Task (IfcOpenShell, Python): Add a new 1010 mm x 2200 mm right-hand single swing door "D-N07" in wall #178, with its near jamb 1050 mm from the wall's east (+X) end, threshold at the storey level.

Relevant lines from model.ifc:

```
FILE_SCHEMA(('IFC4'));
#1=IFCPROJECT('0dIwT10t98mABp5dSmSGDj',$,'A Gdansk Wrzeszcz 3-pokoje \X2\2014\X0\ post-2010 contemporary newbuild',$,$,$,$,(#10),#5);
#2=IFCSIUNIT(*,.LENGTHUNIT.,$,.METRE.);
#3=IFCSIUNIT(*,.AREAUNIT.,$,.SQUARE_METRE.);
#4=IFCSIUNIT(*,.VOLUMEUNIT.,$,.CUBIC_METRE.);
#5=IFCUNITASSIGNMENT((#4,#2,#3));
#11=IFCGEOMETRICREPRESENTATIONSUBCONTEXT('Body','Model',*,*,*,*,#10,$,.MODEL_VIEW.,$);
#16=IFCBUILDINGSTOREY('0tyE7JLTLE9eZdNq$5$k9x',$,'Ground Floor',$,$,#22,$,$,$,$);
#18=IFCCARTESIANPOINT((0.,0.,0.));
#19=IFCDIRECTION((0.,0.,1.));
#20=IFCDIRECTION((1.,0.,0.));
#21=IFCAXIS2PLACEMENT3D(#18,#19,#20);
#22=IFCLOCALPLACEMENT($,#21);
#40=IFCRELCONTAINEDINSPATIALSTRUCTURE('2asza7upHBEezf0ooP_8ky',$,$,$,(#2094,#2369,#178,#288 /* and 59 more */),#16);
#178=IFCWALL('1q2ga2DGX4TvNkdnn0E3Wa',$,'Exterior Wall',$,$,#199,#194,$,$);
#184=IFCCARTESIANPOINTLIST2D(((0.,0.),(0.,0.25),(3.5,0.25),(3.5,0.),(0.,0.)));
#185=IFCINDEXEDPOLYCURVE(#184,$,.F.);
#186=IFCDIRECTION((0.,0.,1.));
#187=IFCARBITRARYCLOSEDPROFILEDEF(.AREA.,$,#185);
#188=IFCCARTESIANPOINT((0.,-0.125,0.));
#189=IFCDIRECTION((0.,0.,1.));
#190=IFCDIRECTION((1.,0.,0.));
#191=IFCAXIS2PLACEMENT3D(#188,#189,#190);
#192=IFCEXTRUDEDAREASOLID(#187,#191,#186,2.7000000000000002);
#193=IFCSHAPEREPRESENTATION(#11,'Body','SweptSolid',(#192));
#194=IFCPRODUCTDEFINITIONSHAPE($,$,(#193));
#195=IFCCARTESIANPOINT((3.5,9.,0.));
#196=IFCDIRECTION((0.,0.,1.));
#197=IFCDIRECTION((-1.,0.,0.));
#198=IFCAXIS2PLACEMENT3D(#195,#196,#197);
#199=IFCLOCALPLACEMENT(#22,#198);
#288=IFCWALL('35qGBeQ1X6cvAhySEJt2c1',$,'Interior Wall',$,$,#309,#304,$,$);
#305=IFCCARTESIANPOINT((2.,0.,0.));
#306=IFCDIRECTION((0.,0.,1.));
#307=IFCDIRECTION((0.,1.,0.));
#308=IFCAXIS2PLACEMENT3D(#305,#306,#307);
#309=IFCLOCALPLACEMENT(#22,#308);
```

```python
import numpy as np
import ifcopenshell
import ifcopenshell.api.feature
import ifcopenshell.api.geometry
import ifcopenshell.api.root
import ifcopenshell.api.spatial
import ifcopenshell.geom
import ifcopenshell.util.element
import ifcopenshell.util.placement
import ifcopenshell.util.representation
import ifcopenshell.util.shape
import ifcopenshell.util.unit

model = ifcopenshell.open("model.ifc")
unit_scale = ifcopenshell.util.unit.calculate_unit_scale(model)
settings = ifcopenshell.geom.settings()


def volume(element):
    """Net volume in cubic metres, openings subtracted."""
    shape = ifcopenshell.geom.create_shape(settings, element)
    return ifcopenshell.util.shape.get_volume(shape.geometry)


wall = model.by_id(178)
storey = ifcopenshell.util.element.get_container(wall, ifc_class="IfcBuildingStorey")
context = ifcopenshell.util.representation.get_context(model, "Model", "Body", "MODEL_VIEW")
before = volume(wall)

width, height, from_end, sill = 1.01, 2.2, 1.05, 0.0  # metres

# The wall runs along its own X axis, and the end named is its -X end.
wall_shape = ifcopenshell.geom.create_shape(settings, wall)
x, y, z = ifcopenshell.util.shape.get_vertices(wall_shape.geometry).T
start = x.min() + from_end
face, thickness = float(y.min()), float(y.max() - y.min())
wall_matrix = ifcopenshell.util.placement.get_local_placement(wall.ObjectPlacement)
level = ifcopenshell.util.placement.get_local_placement(storey.ObjectPlacement)[2, 3]


def in_wall(x, y):
    """Placement at x, y metres in the wall's axes, at sill height."""
    matrix = wall_matrix.copy()
    matrix[:, 3] = wall_matrix @ np.array([x / unit_scale, y / unit_scale, 0.0, 1.0])
    matrix[2, 3] = level + sill / unit_scale
    return matrix


# Opening: a box that overshoots both wall faces by 50 mm.
opening = ifcopenshell.api.root.create_entity(model, ifc_class="IfcOpeningElement", predefined_type="OPENING")
box = ifcopenshell.api.geometry.add_wall_representation(
    model, context=context, length=width, height=height, thickness=thickness + 0.1
)
ifcopenshell.api.geometry.assign_representation(model, product=opening, representation=box)
ifcopenshell.api.geometry.edit_object_placement(model, product=opening, matrix=in_wall(start, face - 0.05), is_si=False)
ifcopenshell.api.feature.add_feature(model, feature=opening, element=wall)

door = ifcopenshell.api.root.create_entity(model, ifc_class="IfcDoor", name="D-N07", predefined_type="DOOR")
door.OverallWidth, door.OverallHeight = width / unit_scale, height / unit_scale
door.OperationType = "SINGLE_SWING_RIGHT"
body = ifcopenshell.api.geometry.add_door_representation(
    model,
    context=context,
    overall_width=door.OverallWidth,
    overall_height=door.OverallHeight,
    operation_type="SINGLE_SWING_RIGHT",
    lining_properties={"LiningDepth": thickness / unit_scale, "ThresholdDepth": thickness / unit_scale},
)
ifcopenshell.api.geometry.assign_representation(model, product=door, representation=body)
ifcopenshell.api.spatial.assign_container(model, products=[door], relating_structure=storey)
ifcopenshell.api.feature.add_filling(model, opening=opening, element=door)

# The lining spans the wall, so the door starts at the wall face.
ifcopenshell.api.geometry.edit_object_placement(model, product=door, matrix=in_wall(start, face), is_si=False)

after = volume(wall)

print(f"wall volume {before:.3f} -> {after:.3f} m3")

model.write("model_rev.ifc")
```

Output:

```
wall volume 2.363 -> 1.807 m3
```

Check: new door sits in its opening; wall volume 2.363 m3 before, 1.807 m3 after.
